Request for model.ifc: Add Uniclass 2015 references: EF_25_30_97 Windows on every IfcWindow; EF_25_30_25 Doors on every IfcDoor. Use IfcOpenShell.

First a look at what the model holds.

```python
import ifcopenshell

model = ifcopenshell.open("model.ifc")
print(model.schema)
print("classifications:", [c.Name for c in model.by_type("IfcClassification")])
for ifc_class in ("IfcDoor", "IfcRoof", "IfcStair", "IfcWall", "IfcWindow"):
    print(ifc_class, len(model.by_type(ifc_class)))
```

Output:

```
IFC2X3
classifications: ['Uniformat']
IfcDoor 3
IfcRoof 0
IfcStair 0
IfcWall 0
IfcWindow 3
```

```python
import ifcopenshell
import ifcopenshell.api.classification

model = ifcopenshell.open("model.ifc")

# IFC2X3 requires Source and Edition and has no link from the project to the system.
system = model.create_entity("IfcClassification", Source="NBS", Edition="2015", Name="Uniclass 2015")

codes = {
    "IfcWindow": ("EF_25_30_97", "Windows"),
    "IfcDoor": ("EF_25_30_25", "Doors"),
}
for ifc_class, (code, name) in codes.items():
    products = model.by_type(ifc_class)
    ifcopenshell.api.classification.add_reference(
        model, products=products, classification=system, identification=code, name=name
    )
    print(code, len(products))

model.write("model-out.ifc")
```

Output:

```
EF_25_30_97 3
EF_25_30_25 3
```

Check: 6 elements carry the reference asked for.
